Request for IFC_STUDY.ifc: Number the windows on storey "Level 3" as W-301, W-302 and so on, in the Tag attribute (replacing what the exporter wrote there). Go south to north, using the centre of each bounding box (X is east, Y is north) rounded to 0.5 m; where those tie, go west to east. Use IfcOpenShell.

First a look at what the model holds.

```python
import ifcopenshell
import ifcopenshell.util.element
import ifcopenshell.util.placement

model = ifcopenshell.open("IFC_STUDY.ifc")
print(model.schema)
storey = next(s for s in model.by_type("IfcBuildingStorey") if s.Name == "Level 3")
windows = [e for e in ifcopenshell.util.element.get_decomposition(storey) if e.is_a("IfcWindow")]
for e in sorted(windows, key=lambda e: e.id()):
    origin = ifcopenshell.util.placement.get_local_placement(e.ObjectPlacement)[:3, 3]
    print(e.id(), e.Tag, e.Name, origin.round(2) + 0.0, sep=" | ")
```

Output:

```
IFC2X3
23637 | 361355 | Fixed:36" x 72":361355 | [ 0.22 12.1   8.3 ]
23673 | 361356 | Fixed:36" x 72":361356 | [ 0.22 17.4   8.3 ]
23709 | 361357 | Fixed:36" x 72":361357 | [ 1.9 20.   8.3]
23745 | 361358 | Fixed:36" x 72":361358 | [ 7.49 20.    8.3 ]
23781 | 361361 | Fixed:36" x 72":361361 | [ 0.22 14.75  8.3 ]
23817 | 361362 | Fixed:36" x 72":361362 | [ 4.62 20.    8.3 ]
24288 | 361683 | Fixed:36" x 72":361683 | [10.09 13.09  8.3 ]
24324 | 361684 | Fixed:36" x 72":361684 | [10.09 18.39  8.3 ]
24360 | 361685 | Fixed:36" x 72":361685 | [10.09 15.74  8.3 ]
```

```python
import ifcopenshell
import ifcopenshell.geom
import ifcopenshell.util.element
import ifcopenshell.util.shape

model = ifcopenshell.open("IFC_STUDY.ifc")
settings = ifcopenshell.geom.settings()
settings.set("use-world-coords", True)


def centre(element):
    shape = ifcopenshell.geom.create_shape(settings, element)
    return ifcopenshell.util.shape.get_bbox_centroid(shape.geometry)


storey = next(s for s in model.by_type("IfcBuildingStorey") if s.Name == "Level 3")
windows = [e for e in ifcopenshell.util.element.get_decomposition(storey) if e.is_a("IfcWindow")]

# Insertion points can sit at a corner or the storey origin, so sort by the geometry (in metres).
centres = {e: centre(e) for e in windows}
windows.sort(key=lambda e: (round(centres[e][1] / 0.5), centres[e][0]))

for i, e in enumerate(windows, start=1):
    number = f"W-3{i:02d}"
    e.Tag = number
    print(e.id(), number)

model.write("IFC_STUDY_v2.ifc")
```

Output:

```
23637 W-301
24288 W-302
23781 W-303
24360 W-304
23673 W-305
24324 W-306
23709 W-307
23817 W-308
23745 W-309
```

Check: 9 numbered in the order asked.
